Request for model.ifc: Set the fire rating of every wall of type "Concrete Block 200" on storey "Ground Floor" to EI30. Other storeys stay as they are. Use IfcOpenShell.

First a look at what the model holds.

```python
import ifcopenshell
import ifcopenshell.util.element

model = ifcopenshell.open("model.ifc")
print(model.schema)
storey = next(s for s in model.by_type("IfcBuildingStorey") if s.Name == "Ground Floor")
walls = [e for e in ifcopenshell.util.element.get_decomposition(storey) if e.is_a("IfcWall")]
seen = {}
for e in walls:
    element_type = ifcopenshell.util.element.get_type(e)
    key = (element_type.Name if element_type != e and element_type else None, ifcopenshell.util.element.get_pset(e, "Pset_WallCommon", "FireRating"))
    seen[key] = seen.get(key, 0) + 1
for (name, value), count in sorted(seen.items(), key=str):
    print(count, "x", name, "|", value)
```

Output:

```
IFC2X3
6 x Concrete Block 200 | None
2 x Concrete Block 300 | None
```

```python
import ifcopenshell
import ifcopenshell.api.pset
import ifcopenshell.util.element

model = ifcopenshell.open("model.ifc")

storey = next(s for s in model.by_type("IfcBuildingStorey") if s.Name == "Ground Floor")
walls = [e for e in ifcopenshell.util.element.get_decomposition(storey) if e.is_a("IfcWall")]

count = 0
for e in walls:
    element_type = ifcopenshell.util.element.get_type(e)
    if element_type in (None, e) or element_type.Name != "Concrete Block 200":
        continue
    # add_pset returns the element's existing set when there is one.
    pset = ifcopenshell.api.pset.add_pset(model, product=e, name="Pset_WallCommon")
    ifcopenshell.api.pset.edit_pset(model, pset=pset, properties={"FireRating": "EI30"})
    count += 1

print(count, "walls updated")

model.write("model_updated.ifc")
```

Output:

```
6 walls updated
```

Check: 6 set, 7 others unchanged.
